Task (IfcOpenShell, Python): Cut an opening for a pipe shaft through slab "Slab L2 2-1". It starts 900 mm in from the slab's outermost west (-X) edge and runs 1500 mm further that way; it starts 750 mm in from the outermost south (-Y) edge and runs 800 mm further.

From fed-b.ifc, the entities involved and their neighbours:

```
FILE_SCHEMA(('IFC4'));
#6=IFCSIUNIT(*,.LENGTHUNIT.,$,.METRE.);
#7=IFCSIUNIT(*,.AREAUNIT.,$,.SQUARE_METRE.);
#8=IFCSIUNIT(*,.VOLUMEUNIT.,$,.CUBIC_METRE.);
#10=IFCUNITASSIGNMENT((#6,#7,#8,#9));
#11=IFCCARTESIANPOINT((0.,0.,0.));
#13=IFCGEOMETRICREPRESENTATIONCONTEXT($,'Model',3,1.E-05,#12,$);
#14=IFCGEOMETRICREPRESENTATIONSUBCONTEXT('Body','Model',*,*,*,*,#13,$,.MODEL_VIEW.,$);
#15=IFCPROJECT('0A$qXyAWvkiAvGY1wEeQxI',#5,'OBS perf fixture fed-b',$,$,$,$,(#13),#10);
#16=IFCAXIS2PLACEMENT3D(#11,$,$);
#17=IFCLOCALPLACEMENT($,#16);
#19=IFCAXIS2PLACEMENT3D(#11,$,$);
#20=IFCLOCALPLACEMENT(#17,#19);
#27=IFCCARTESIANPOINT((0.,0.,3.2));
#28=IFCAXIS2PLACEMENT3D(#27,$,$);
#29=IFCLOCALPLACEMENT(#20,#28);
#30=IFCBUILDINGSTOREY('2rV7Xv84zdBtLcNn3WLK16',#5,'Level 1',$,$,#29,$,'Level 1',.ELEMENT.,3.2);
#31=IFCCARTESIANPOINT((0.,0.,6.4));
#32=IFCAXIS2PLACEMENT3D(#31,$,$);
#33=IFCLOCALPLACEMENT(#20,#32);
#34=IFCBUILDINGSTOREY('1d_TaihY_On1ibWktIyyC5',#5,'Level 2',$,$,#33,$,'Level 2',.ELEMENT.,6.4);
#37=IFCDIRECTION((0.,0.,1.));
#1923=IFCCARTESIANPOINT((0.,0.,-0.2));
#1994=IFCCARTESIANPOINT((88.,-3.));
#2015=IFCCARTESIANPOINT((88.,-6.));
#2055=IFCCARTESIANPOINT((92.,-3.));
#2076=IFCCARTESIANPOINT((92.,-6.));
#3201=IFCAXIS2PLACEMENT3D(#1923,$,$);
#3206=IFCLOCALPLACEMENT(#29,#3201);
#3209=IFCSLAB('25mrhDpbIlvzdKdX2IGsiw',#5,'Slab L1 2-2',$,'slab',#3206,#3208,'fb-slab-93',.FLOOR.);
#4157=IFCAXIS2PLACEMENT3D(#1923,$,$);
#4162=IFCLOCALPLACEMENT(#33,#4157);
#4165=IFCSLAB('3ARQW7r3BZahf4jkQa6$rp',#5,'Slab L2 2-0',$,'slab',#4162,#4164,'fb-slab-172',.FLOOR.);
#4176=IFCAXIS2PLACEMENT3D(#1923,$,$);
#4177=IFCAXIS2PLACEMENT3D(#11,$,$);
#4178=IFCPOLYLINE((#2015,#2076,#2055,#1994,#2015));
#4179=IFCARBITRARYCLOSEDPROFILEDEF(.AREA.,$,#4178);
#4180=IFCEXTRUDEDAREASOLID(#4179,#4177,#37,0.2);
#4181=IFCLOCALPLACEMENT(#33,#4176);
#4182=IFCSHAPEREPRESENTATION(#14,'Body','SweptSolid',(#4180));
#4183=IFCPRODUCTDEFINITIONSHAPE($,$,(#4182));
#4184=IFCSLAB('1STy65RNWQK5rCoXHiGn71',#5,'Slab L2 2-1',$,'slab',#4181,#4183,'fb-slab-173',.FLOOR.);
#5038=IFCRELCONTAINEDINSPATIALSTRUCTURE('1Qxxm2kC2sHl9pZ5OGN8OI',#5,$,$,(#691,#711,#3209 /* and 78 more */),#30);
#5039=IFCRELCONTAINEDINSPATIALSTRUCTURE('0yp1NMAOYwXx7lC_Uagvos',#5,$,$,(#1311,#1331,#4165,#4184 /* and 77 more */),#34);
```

```python
import numpy as np
import ifcopenshell
import ifcopenshell.api.feature
import ifcopenshell.api.geometry
import ifcopenshell.api.root
import ifcopenshell.geom
import ifcopenshell.util.placement
import ifcopenshell.util.representation
import ifcopenshell.util.shape
import ifcopenshell.util.unit

model = ifcopenshell.open("fed-b.ifc")
unit_scale = ifcopenshell.util.unit.calculate_unit_scale(model)
settings = ifcopenshell.geom.settings()


def volume(element):
    """Net volume in cubic metres, openings subtracted."""
    shape = ifcopenshell.geom.create_shape(settings, element)
    return ifcopenshell.util.shape.get_volume(shape.geometry)


slab = model.by_guid("1STy65RNWQK5rCoXHiGn71")
before = volume(slab)

# Extent in the slab's own axes, in metres. The edges named are its -X and -Y sides.
slab_shape = ifcopenshell.geom.create_shape(settings, slab)
vertices = ifcopenshell.util.shape.get_vertices(slab_shape.geometry)
x_min, y_min, bottom = vertices.min(axis=0)
top = vertices[:, 2].max()

opening = ifcopenshell.api.root.create_entity(model, ifc_class="IfcOpeningElement", name="Pipe shaft opening", predefined_type="OPENING")
context = ifcopenshell.util.representation.get_context(model, "Model", "Body", "MODEL_VIEW")
width, depth = 1.5, 0.8
outline = [(0.0, 0.0), (width, 0.0), (width, depth), (0.0, depth), (0.0, 0.0)]
# Overshoot both faces by 50 mm so the cut is clean.
shape = ifcopenshell.api.geometry.add_slab_representation(
    model, context=context, depth=top - bottom + 0.1, polyline=outline
)
ifcopenshell.api.geometry.assign_representation(model, product=opening, representation=shape)

matrix = ifcopenshell.util.placement.get_local_placement(slab.ObjectPlacement)
matrix[:, 3] = matrix @ np.append(np.array([x_min + 0.9, y_min + 0.75, bottom - 0.05]) / unit_scale, 1.0)
ifcopenshell.api.geometry.edit_object_placement(model, product=opening, matrix=matrix, is_si=False)
ifcopenshell.api.feature.add_feature(model, feature=opening, element=slab)

after = volume(slab)

print(f"slab volume {before:.3f} -> {after:.3f} m3")

model.write("fed-b_updated.ifc")
```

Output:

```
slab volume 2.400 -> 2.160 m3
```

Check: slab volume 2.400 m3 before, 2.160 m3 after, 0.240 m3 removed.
